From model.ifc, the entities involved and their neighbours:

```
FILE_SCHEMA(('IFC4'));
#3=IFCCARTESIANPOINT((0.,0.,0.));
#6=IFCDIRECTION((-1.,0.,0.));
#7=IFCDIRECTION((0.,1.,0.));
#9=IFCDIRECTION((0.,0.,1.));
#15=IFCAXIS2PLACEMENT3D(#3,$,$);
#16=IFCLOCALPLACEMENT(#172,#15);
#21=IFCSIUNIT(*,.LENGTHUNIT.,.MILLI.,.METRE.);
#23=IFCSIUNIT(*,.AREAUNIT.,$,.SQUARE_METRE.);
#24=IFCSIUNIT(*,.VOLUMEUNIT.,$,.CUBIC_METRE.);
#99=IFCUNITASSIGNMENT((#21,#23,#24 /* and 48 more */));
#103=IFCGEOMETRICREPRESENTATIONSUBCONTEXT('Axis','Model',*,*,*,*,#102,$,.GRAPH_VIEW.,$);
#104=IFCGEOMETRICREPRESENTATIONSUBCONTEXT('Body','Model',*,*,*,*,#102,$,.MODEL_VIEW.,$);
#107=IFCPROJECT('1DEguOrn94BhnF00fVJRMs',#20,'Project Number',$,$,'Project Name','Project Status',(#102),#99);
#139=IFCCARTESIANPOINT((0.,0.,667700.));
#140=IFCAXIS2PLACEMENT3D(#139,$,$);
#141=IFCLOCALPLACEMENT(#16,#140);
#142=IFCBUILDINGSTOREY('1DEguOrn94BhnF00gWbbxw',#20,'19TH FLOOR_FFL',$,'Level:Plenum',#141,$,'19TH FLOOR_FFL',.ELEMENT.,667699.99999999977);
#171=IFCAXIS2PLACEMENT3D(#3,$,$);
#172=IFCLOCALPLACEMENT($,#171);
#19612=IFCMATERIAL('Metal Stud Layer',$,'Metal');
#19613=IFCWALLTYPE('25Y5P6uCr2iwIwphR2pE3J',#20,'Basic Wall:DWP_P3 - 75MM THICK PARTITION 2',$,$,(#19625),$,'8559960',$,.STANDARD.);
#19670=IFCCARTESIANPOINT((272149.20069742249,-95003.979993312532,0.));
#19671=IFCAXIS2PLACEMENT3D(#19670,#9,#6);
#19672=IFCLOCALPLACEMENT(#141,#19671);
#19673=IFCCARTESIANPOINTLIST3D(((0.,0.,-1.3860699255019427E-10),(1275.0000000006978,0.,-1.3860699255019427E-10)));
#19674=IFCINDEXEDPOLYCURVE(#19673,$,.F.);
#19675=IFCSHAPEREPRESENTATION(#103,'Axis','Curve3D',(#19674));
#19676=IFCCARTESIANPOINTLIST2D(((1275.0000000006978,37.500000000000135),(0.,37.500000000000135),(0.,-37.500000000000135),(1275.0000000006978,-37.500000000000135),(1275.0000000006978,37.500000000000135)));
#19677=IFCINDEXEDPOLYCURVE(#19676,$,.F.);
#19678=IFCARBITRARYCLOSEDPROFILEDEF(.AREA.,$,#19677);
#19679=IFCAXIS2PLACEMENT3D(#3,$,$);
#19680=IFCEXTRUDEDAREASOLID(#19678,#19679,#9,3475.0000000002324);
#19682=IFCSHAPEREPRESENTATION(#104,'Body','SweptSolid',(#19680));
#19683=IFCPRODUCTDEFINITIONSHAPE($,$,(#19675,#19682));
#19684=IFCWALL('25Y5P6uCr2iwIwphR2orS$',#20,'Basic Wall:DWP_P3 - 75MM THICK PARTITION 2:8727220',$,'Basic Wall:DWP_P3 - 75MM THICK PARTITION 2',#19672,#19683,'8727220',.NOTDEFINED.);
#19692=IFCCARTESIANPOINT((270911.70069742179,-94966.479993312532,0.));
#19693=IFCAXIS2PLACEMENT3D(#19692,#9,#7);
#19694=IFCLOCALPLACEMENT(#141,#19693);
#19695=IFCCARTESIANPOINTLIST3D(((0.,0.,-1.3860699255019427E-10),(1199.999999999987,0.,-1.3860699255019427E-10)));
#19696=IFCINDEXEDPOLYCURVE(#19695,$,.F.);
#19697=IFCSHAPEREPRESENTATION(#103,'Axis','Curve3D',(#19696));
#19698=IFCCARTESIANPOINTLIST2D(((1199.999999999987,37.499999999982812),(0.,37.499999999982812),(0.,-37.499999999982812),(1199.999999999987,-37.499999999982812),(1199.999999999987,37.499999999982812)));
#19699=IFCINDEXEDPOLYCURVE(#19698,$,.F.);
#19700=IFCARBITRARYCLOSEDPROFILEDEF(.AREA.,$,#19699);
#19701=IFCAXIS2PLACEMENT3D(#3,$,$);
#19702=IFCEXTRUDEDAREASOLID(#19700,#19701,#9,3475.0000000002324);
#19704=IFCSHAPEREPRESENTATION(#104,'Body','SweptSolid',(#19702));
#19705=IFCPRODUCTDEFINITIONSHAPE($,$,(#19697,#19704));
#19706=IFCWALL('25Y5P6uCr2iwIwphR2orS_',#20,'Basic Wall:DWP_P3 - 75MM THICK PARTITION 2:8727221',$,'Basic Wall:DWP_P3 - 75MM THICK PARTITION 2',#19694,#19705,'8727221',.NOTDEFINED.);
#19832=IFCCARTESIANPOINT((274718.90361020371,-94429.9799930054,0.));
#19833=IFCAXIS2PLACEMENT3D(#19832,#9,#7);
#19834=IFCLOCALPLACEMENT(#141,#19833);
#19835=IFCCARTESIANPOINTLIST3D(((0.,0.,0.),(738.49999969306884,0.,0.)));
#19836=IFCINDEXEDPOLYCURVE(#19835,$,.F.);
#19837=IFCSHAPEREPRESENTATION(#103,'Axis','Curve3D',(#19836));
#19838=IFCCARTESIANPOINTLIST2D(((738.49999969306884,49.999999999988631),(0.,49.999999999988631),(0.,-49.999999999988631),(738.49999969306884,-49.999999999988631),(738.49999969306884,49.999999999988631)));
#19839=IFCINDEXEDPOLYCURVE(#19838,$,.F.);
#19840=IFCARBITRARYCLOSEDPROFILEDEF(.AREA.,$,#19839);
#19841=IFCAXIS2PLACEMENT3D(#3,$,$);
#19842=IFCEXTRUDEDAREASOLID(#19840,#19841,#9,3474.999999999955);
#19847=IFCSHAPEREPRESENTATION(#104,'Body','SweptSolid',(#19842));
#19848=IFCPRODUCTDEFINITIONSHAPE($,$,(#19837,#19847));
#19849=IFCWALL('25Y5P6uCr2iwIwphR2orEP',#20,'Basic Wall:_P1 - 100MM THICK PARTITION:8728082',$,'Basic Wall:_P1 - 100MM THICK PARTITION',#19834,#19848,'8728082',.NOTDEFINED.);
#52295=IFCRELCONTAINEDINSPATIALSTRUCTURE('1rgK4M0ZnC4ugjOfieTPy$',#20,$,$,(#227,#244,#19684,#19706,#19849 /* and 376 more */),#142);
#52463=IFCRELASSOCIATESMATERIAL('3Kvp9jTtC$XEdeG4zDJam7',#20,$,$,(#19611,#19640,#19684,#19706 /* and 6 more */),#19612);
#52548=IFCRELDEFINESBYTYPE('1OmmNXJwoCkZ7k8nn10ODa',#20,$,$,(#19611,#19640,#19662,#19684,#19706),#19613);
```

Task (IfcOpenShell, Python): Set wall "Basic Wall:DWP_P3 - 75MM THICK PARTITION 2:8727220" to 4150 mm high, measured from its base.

```python
import ifcopenshell
import ifcopenshell.geom
import ifcopenshell.util.representation
import ifcopenshell.util.shape

model = ifcopenshell.open("model.ifc")
settings = ifcopenshell.geom.settings()


def volume(element):
    """Net volume in cubic metres, openings subtracted."""
    shape = ifcopenshell.geom.create_shape(settings, element)
    return ifcopenshell.util.shape.get_volume(shape.geometry)


wall = model.by_id(19684)
before = volume(wall)

body = ifcopenshell.util.representation.get_representation(wall, "Model", "Body")
solid = body.Items[0]
old_height = solid.Depth
solid.Depth = 4150.0
after = volume(wall)

print(f"height {old_height:g} -> {solid.Depth:g}, volume {before:.3f} -> {after:.3f} m3")

model.write("model_v2.ifc")
```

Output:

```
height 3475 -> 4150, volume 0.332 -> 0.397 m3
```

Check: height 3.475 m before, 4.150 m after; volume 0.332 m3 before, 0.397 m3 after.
